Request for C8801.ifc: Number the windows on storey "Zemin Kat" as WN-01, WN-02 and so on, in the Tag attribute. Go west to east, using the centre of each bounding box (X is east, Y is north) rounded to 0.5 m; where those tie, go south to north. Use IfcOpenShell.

First a look at what the model holds.

```python
import ifcopenshell
import ifcopenshell.util.element
import ifcopenshell.util.placement

model = ifcopenshell.open("C8801.ifc")
print(model.schema)
storey = next(s for s in model.by_type("IfcBuildingStorey") if s.Name == "Zemin Kat")
windows = [e for e in ifcopenshell.util.element.get_decomposition(storey) if e.is_a("IfcWindow")]
for e in sorted(windows, key=lambda e: e.id()):
    origin = ifcopenshell.util.placement.get_local_placement(e.ObjectPlacement)[:3, 3]
    print(e.id(), e.Tag, e.Name, origin.round(2) + 0.0, sep=" | ")
```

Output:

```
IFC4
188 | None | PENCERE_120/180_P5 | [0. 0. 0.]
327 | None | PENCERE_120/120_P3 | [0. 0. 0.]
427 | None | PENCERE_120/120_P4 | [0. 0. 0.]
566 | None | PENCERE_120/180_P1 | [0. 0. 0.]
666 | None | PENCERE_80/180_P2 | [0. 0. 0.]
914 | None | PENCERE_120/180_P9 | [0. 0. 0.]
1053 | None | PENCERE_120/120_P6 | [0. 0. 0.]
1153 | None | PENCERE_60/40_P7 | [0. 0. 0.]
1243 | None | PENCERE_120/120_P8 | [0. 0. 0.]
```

```python
import ifcopenshell
import ifcopenshell.geom
import ifcopenshell.util.element
import ifcopenshell.util.shape

model = ifcopenshell.open("C8801.ifc")
settings = ifcopenshell.geom.settings()
settings.set("use-world-coords", True)


def centre(element):
    shape = ifcopenshell.geom.create_shape(settings, element)
    return ifcopenshell.util.shape.get_bbox_centroid(shape.geometry)


storey = next(s for s in model.by_type("IfcBuildingStorey") if s.Name == "Zemin Kat")
windows = [e for e in ifcopenshell.util.element.get_decomposition(storey) if e.is_a("IfcWindow")]

# Insertion points can sit at a corner or the storey origin, so sort by the geometry (in metres).
centres = {e: centre(e) for e in windows}
windows.sort(key=lambda e: (round(centres[e][0] / 0.5), centres[e][1]))

for i, e in enumerate(windows, start=1):
    number = f"WN-{i:02d}"
    e.Tag = number
    print(e.id(), number)

model.write("C8801-out.ifc")
```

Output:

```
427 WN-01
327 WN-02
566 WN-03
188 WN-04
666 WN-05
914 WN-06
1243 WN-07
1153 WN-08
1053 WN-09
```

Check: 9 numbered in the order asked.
